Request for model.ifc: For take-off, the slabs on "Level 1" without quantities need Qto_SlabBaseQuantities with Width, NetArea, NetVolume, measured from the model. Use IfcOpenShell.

First a look at what the model holds.

```python
import ifcopenshell
import ifcopenshell.util.element
import ifcopenshell.util.unit

model = ifcopenshell.open("model.ifc")
print(model.schema)
for unit_type in ("LENGTHUNIT", "AREAUNIT", "VOLUMEUNIT"):
    print(unit_type, ifcopenshell.util.unit.calculate_unit_scale(model, unit_type))
storey = next(s for s in model.by_type("IfcBuildingStorey") if s.Name == "Level 1")
slabs = [e for e in ifcopenshell.util.element.get_decomposition(storey) if e.is_a("IfcSlab")]
for e in sorted(slabs, key=lambda e: e.id()):
    print(e.id(), e.is_a(), e.Name, list(ifcopenshell.util.element.get_psets(e, qtos_only=True)), sep=" | ")
```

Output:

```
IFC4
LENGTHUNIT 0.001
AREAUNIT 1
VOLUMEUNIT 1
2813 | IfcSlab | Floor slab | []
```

```python
import ifcopenshell
import ifcopenshell.api.pset
import ifcopenshell.geom
import ifcopenshell.util.element
import ifcopenshell.util.shape
import ifcopenshell.util.unit

model = ifcopenshell.open("model.ifc")
unit_scale = ifcopenshell.util.unit.calculate_unit_scale(model)
area_scale = ifcopenshell.util.unit.calculate_unit_scale(model, "AREAUNIT")
volume_scale = ifcopenshell.util.unit.calculate_unit_scale(model, "VOLUMEUNIT")
settings = ifcopenshell.geom.settings()

storey = next(s for s in model.by_type("IfcBuildingStorey") if s.Name == "Level 1")
slabs = [e for e in ifcopenshell.util.element.get_decomposition(storey) if e.is_a("IfcSlab")]

for e in sorted(slabs, key=lambda e: e.id()):
    if ifcopenshell.util.element.get_psets(e, qtos_only=True, should_inherit=False):
        continue
    # Geometry comes back in metres, in the element's own axes.
    shape = ifcopenshell.geom.create_shape(settings, e)
    values = {
        "Width": ifcopenshell.util.shape.get_z(shape.geometry) / unit_scale,
        "NetArea": ifcopenshell.util.shape.get_footprint_area(shape.geometry) / area_scale,
        "NetVolume": ifcopenshell.util.shape.get_volume(shape.geometry) / volume_scale,
    }
    qto = ifcopenshell.api.pset.add_qto(model, product=e, name="Qto_SlabBaseQuantities")
    ifcopenshell.api.pset.edit_qto(model, qto=qto, properties=values)
    print(e.id(), {k: round(v, 3) for k, v in values.items()})

model.write("model-out.ifc")
```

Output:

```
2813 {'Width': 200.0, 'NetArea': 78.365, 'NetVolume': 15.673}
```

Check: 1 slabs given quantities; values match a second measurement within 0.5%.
